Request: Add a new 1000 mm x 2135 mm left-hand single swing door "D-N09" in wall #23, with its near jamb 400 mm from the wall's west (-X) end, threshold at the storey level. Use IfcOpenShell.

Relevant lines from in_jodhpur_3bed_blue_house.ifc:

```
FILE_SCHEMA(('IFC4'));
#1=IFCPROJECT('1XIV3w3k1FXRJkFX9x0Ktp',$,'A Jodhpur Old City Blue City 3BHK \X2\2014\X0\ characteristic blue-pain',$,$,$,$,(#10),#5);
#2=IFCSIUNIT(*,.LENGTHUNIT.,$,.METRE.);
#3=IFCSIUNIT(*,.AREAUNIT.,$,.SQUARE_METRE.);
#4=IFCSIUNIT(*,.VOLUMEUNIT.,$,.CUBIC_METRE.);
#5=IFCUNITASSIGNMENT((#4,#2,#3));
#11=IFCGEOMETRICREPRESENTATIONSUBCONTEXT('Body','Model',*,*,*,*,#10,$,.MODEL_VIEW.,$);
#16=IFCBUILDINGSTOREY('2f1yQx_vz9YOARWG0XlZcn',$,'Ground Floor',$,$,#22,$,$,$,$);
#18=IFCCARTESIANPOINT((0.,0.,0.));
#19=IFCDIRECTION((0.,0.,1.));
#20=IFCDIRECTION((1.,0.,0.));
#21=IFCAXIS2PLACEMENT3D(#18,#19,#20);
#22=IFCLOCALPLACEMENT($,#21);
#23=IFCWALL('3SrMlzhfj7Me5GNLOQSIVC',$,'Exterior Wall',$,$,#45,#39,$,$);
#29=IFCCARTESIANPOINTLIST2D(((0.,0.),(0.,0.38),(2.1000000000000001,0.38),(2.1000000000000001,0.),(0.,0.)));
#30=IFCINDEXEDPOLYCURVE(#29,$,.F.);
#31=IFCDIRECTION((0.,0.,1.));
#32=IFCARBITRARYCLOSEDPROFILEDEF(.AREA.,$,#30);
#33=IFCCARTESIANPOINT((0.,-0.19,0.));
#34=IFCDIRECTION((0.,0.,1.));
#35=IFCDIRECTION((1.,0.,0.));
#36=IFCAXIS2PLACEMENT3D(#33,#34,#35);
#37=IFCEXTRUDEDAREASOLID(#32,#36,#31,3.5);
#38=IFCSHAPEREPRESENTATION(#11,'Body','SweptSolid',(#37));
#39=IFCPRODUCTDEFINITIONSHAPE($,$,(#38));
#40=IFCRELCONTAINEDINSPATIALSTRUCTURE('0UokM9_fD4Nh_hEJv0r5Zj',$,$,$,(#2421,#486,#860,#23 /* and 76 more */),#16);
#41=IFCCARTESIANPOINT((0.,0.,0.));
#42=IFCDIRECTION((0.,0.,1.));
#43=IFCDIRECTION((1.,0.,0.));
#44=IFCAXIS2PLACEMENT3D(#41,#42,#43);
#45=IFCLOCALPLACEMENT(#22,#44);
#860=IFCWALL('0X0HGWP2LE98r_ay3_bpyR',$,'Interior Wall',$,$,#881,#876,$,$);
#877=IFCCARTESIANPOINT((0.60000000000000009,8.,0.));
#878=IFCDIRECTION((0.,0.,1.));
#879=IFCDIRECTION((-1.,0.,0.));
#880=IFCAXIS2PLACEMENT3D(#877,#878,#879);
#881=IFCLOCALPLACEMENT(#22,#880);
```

```python
import numpy as np
import ifcopenshell
import ifcopenshell.api.feature
import ifcopenshell.api.geometry
import ifcopenshell.api.root
import ifcopenshell.api.spatial
import ifcopenshell.geom
import ifcopenshell.util.element
import ifcopenshell.util.placement
import ifcopenshell.util.representation
import ifcopenshell.util.shape
import ifcopenshell.util.unit

model = ifcopenshell.open("in_jodhpur_3bed_blue_house.ifc")
unit_scale = ifcopenshell.util.unit.calculate_unit_scale(model)
settings = ifcopenshell.geom.settings()


def volume(element):
    """Net volume in cubic metres, openings subtracted."""
    shape = ifcopenshell.geom.create_shape(settings, element)
    return ifcopenshell.util.shape.get_volume(shape.geometry)


wall = model.by_id(23)
storey = ifcopenshell.util.element.get_container(wall, ifc_class="IfcBuildingStorey")
context = ifcopenshell.util.representation.get_context(model, "Model", "Body", "MODEL_VIEW")
before = volume(wall)

width, height, from_end, sill = 1, 2.135, 0.4, 0.0  # metres

# The wall runs along its own X axis, and the end named is its -X end.
wall_shape = ifcopenshell.geom.create_shape(settings, wall)
x, y, z = ifcopenshell.util.shape.get_vertices(wall_shape.geometry).T
start = x.min() + from_end
face, thickness = float(y.min()), float(y.max() - y.min())
wall_matrix = ifcopenshell.util.placement.get_local_placement(wall.ObjectPlacement)
level = ifcopenshell.util.placement.get_local_placement(storey.ObjectPlacement)[2, 3]


def in_wall(x, y):
    """Placement at x, y metres in the wall's axes, at sill height."""
    matrix = wall_matrix.copy()
    matrix[:, 3] = wall_matrix @ np.array([x / unit_scale, y / unit_scale, 0.0, 1.0])
    matrix[2, 3] = level + sill / unit_scale
    return matrix


# Opening: a box that overshoots both wall faces by 50 mm.
opening = ifcopenshell.api.root.create_entity(model, ifc_class="IfcOpeningElement", predefined_type="OPENING")
box = ifcopenshell.api.geometry.add_wall_representation(
    model, context=context, length=width, height=height, thickness=thickness + 0.1
)
ifcopenshell.api.geometry.assign_representation(model, product=opening, representation=box)
ifcopenshell.api.geometry.edit_object_placement(model, product=opening, matrix=in_wall(start, face - 0.05), is_si=False)
ifcopenshell.api.feature.add_feature(model, feature=opening, element=wall)

door = ifcopenshell.api.root.create_entity(model, ifc_class="IfcDoor", name="D-N09", predefined_type="DOOR")
door.OverallWidth, door.OverallHeight = width / unit_scale, height / unit_scale
door.OperationType = "SINGLE_SWING_LEFT"
body = ifcopenshell.api.geometry.add_door_representation(
    model,
    context=context,
    overall_width=door.OverallWidth,
    overall_height=door.OverallHeight,
    operation_type="SINGLE_SWING_LEFT",
    lining_properties={"LiningDepth": thickness / unit_scale, "ThresholdDepth": thickness / unit_scale},
)
ifcopenshell.api.geometry.assign_representation(model, product=door, representation=body)
ifcopenshell.api.spatial.assign_container(model, products=[door], relating_structure=storey)
ifcopenshell.api.feature.add_filling(model, opening=opening, element=door)

# The lining spans the wall, so the door starts at the wall face.
ifcopenshell.api.geometry.edit_object_placement(model, product=door, matrix=in_wall(start, face), is_si=False)

after = volume(wall)

print(f"wall volume {before:.3f} -> {after:.3f} m3")

model.write("in_jodhpur_3bed_blue_house_updated.ifc")
```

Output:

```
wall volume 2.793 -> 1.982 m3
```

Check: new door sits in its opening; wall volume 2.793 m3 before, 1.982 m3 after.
